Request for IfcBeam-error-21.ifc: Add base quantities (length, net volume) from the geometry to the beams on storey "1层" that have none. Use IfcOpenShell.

First a look at what the model holds.

```python
import ifcopenshell
import ifcopenshell.util.element
import ifcopenshell.util.unit

model = ifcopenshell.open("IfcBeam-error-21.ifc")
print(model.schema)
for unit_type in ("LENGTHUNIT", "AREAUNIT", "VOLUMEUNIT"):
    print(unit_type, ifcopenshell.util.unit.calculate_unit_scale(model, unit_type))
storey = next(s for s in model.by_type("IfcBuildingStorey") if s.Name == "1层")
beams = [e for e in ifcopenshell.util.element.get_decomposition(storey) if e.is_a("IfcBeam")]
for e in sorted(beams, key=lambda e: e.id()):
    print(e.id(), e.is_a(), e.Name, list(ifcopenshell.util.element.get_psets(e, qtos_only=True)), sep=" | ")
```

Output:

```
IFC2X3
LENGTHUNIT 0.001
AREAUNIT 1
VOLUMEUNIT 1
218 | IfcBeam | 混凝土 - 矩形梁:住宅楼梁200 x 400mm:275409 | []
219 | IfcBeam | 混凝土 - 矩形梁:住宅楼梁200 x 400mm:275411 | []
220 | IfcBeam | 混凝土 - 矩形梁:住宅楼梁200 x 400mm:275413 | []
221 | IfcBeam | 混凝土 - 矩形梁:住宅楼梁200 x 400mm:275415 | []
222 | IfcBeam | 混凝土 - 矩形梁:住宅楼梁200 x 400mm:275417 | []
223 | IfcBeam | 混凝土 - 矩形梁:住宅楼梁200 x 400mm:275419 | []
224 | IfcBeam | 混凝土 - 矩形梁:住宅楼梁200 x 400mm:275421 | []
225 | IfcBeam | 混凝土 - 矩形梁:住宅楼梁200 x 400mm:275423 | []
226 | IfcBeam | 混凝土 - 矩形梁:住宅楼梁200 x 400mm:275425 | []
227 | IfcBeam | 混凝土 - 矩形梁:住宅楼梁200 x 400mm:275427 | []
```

```python
import ifcopenshell
import ifcopenshell.api.pset
import ifcopenshell.geom
import ifcopenshell.util.element
import ifcopenshell.util.shape
import ifcopenshell.util.unit

model = ifcopenshell.open("IfcBeam-error-21.ifc")
unit_scale = ifcopenshell.util.unit.calculate_unit_scale(model)
volume_scale = ifcopenshell.util.unit.calculate_unit_scale(model, "VOLUMEUNIT")
settings = ifcopenshell.geom.settings()

storey = next(s for s in model.by_type("IfcBuildingStorey") if s.Name == "1层")
beams = [e for e in ifcopenshell.util.element.get_decomposition(storey) if e.is_a("IfcBeam")]

for e in sorted(beams, key=lambda e: e.id()):
    if ifcopenshell.util.element.get_psets(e, qtos_only=True, should_inherit=False):
        continue
    # Geometry comes back in metres, in the element's own axes.
    shape = ifcopenshell.geom.create_shape(settings, e)
    values = {
        "Length": ifcopenshell.util.shape.get_max_xyz(shape.geometry) / unit_scale,
        "NetVolume": ifcopenshell.util.shape.get_volume(shape.geometry) / volume_scale,
    }
    qto = ifcopenshell.api.pset.add_qto(model, product=e, name="BaseQuantities")
    ifcopenshell.api.pset.edit_qto(model, qto=qto, properties=values)
    print(e.id(), {k: round(v, 3) for k, v in values.items()})

model.write("IfcBeam-error-21_edited.ifc")
```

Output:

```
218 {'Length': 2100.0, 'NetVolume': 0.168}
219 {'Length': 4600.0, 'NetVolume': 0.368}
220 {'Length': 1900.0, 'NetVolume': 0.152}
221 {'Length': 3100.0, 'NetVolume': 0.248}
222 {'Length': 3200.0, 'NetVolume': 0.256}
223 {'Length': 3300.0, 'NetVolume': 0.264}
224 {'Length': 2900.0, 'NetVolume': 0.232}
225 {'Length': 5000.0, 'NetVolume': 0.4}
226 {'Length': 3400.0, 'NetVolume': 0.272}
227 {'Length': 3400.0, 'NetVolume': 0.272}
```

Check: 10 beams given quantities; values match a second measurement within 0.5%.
